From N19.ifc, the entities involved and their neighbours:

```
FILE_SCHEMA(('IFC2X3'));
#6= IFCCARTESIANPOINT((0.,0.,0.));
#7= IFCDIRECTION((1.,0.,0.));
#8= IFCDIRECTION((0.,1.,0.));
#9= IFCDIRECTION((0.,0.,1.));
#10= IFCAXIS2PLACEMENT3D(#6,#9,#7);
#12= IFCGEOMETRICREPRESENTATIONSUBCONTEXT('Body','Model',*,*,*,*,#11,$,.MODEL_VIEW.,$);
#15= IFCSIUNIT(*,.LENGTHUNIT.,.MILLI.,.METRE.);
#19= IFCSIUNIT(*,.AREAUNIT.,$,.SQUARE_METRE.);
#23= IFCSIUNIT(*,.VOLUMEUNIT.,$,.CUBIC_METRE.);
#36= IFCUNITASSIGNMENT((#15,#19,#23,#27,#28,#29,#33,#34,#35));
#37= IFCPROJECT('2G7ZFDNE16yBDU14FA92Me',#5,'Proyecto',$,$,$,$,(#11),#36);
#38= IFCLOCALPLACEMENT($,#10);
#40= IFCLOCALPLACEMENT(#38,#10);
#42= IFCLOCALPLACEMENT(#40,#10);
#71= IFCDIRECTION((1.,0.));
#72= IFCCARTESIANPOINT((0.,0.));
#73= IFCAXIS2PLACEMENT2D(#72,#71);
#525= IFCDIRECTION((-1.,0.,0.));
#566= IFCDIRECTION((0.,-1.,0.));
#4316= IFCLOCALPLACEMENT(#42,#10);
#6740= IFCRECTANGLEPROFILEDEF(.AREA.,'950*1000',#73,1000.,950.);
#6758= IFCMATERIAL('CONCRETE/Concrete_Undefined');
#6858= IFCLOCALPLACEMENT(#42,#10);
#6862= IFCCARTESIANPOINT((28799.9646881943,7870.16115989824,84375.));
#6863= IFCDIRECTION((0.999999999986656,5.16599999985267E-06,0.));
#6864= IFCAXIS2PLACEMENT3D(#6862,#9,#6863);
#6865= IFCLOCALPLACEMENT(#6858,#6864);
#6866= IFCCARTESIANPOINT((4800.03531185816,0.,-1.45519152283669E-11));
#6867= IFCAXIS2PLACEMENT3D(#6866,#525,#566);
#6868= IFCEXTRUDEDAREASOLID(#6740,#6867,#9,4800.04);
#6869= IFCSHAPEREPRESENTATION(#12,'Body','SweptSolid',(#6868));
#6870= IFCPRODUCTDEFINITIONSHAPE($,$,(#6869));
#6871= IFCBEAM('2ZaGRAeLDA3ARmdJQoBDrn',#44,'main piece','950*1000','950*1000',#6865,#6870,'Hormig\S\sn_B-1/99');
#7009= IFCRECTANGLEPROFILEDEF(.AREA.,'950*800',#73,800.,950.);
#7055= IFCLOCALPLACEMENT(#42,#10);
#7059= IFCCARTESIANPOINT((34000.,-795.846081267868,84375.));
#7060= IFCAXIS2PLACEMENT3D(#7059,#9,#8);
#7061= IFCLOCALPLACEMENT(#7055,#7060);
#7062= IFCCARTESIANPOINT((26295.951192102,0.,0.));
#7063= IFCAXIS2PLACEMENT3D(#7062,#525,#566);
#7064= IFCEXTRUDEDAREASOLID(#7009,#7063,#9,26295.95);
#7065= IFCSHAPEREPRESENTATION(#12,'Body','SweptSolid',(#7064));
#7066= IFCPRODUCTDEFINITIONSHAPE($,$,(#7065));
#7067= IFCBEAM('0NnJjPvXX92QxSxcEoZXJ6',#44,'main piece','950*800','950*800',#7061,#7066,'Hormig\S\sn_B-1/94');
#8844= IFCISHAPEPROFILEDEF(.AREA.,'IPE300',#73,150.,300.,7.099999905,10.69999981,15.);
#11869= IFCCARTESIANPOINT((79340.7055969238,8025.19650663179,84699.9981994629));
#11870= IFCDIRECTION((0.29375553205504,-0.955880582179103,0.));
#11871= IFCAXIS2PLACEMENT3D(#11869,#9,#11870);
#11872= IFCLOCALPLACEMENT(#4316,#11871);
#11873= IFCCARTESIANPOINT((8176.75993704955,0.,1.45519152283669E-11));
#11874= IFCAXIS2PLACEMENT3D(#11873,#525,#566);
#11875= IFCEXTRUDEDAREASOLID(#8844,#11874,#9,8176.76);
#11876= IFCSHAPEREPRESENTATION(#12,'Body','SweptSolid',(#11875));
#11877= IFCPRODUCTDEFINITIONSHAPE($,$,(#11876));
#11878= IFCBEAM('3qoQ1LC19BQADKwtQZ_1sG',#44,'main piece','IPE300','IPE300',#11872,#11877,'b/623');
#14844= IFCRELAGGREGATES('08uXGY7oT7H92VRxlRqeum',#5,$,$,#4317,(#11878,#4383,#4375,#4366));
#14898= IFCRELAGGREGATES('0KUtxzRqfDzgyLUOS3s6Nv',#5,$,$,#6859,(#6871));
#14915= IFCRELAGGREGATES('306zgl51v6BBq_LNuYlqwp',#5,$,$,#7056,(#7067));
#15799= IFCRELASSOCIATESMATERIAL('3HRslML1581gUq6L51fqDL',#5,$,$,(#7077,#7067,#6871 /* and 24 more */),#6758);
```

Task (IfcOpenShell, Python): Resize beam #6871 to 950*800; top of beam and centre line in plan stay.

```python
import ifcopenshell
import ifcopenshell.util.element
import ifcopenshell.util.representation

model = ifcopenshell.open("N19.ifc")

member = model.by_guid("2ZaGRAeLDA3ARmdJQoBDrn")
source = next(p for p in model.by_type("IfcRectangleProfileDef") if p.ProfileName == "950*800")

body = ifcopenshell.util.representation.get_representation(member, "Model", "Body")
solid = body.Items[0]
old_profile = solid.SweptArea

# Copy the section's sizes but keep this member's own profile position.
profile = ifcopenshell.util.element.copy(model, source)
# Profiles are centred, so shift by half the change in depth to hold the top.
shift = (old_profile.YDim - profile.YDim) / 2
x, y = old_profile.Position.Location.Coordinates
up = (0.0, 1.0)  # upwards, in the solid's own plane
location = model.createIfcCartesianPoint((x + up[0] * shift, y + up[1] * shift))
profile.Position = model.createIfcAxis2Placement2D(location, old_profile.Position.RefDirection)
solid.SweptArea = profile
if not model.get_total_inverses(old_profile):
    ifcopenshell.util.element.remove_deep2(model, old_profile)
member.Description = member.Description.replace("950*1000", "950*800")
member.ObjectType = member.ObjectType.replace("950*1000", "950*800")

print(solid.SweptArea)

model.write("N19_edited.ifc")
```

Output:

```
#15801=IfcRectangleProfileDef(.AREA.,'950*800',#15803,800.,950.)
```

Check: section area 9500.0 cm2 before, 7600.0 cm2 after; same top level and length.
